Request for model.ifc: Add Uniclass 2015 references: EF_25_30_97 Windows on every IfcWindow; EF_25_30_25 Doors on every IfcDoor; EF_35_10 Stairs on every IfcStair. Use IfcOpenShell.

First a look at what the model holds.

```python
import ifcopenshell

model = ifcopenshell.open("model.ifc")
print(model.schema)
print("classifications:", [c.Name for c in model.by_type("IfcClassification")])
for ifc_class in ("IfcDoor", "IfcRoof", "IfcStair", "IfcWall", "IfcWindow"):
    print(ifc_class, len(model.by_type(ifc_class)))
```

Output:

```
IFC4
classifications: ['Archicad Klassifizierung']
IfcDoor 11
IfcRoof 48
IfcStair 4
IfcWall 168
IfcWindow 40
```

```python
import ifcopenshell
import ifcopenshell.api.classification

model = ifcopenshell.open("model.ifc")

system = ifcopenshell.api.classification.add_classification(model, classification="Uniclass 2015")

codes = {
    "IfcWindow": ("EF_25_30_97", "Windows"),
    "IfcDoor": ("EF_25_30_25", "Doors"),
    "IfcStair": ("EF_35_10", "Stairs"),
}
for ifc_class, (code, name) in codes.items():
    products = model.by_type(ifc_class)
    ifcopenshell.api.classification.add_reference(
        model, products=products, classification=system, identification=code, name=name
    )
    print(code, len(products))

model.write("model_v2.ifc")
```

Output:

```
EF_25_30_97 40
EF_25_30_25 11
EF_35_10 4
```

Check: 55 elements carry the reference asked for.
